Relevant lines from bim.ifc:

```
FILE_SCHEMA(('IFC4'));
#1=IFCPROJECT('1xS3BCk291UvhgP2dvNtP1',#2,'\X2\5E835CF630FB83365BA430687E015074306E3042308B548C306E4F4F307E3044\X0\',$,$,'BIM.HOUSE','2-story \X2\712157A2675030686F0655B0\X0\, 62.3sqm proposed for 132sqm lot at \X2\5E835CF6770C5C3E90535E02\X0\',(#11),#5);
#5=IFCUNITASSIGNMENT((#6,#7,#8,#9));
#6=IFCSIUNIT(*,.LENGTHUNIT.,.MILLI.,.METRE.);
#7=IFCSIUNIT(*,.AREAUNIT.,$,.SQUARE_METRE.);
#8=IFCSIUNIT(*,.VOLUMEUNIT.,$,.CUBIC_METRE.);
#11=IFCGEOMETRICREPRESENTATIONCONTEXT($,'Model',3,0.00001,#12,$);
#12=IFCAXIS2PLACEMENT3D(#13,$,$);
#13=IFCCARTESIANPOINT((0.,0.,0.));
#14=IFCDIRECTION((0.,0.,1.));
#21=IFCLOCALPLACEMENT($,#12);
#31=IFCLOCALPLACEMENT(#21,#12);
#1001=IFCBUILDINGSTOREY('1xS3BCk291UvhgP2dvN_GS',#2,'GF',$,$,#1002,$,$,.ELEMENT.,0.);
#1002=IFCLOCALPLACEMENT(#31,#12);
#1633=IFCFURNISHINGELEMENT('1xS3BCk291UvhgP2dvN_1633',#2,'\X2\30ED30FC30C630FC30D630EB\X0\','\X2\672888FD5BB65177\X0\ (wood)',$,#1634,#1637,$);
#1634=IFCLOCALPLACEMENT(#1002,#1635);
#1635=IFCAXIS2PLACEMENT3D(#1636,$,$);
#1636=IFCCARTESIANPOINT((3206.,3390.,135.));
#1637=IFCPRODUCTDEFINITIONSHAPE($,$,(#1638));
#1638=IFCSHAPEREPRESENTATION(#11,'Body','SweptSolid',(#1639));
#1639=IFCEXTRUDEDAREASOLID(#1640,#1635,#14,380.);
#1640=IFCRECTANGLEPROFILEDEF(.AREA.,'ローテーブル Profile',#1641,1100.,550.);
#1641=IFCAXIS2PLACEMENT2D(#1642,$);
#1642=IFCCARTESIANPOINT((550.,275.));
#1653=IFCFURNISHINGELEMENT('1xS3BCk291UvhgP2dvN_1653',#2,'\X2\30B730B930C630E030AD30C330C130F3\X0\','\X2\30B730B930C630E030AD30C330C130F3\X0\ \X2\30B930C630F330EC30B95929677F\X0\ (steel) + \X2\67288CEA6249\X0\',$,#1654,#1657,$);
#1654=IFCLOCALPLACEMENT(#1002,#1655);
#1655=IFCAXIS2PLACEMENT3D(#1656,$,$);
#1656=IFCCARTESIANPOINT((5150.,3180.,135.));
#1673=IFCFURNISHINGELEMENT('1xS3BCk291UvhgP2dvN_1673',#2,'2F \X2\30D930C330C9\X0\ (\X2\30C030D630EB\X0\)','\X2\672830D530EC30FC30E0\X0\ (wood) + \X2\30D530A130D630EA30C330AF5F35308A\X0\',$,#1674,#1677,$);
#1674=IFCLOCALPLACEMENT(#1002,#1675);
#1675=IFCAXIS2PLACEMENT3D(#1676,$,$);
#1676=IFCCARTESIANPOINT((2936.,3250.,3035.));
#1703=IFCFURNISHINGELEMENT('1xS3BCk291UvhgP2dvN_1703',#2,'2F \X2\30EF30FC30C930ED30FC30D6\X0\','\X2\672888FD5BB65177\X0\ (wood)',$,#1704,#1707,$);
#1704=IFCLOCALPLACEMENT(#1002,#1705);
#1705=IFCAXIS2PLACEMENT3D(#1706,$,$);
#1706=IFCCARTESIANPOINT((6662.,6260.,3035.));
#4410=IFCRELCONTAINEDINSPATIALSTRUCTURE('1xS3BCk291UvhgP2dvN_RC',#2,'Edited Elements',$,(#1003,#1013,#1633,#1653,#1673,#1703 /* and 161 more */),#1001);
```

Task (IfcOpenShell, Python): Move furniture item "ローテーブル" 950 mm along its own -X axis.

```python
import ifcopenshell
import ifcopenshell.api.geometry
import ifcopenshell.util.placement
import ifcopenshell.util.unit

model = ifcopenshell.open("bim.ifc")
unit_scale = ifcopenshell.util.unit.calculate_unit_scale(model)

item = model.by_guid("1xS3BCk291UvhgP2dvN_1633")
matrix = ifcopenshell.util.placement.get_local_placement(item.ObjectPlacement)
matrix[:3, 3] -= matrix[:3, 0] * 0.95 / unit_scale
ifcopenshell.api.geometry.edit_object_placement(model, product=item, matrix=matrix, is_si=False)

print(ifcopenshell.util.placement.get_local_placement(item.ObjectPlacement).round(3) + 0.0)

model.write("bim_edited.ifc")
```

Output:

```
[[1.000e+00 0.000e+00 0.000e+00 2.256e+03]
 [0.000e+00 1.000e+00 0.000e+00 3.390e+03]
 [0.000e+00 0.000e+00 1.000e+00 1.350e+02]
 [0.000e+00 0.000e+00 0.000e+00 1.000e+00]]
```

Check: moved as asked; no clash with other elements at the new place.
